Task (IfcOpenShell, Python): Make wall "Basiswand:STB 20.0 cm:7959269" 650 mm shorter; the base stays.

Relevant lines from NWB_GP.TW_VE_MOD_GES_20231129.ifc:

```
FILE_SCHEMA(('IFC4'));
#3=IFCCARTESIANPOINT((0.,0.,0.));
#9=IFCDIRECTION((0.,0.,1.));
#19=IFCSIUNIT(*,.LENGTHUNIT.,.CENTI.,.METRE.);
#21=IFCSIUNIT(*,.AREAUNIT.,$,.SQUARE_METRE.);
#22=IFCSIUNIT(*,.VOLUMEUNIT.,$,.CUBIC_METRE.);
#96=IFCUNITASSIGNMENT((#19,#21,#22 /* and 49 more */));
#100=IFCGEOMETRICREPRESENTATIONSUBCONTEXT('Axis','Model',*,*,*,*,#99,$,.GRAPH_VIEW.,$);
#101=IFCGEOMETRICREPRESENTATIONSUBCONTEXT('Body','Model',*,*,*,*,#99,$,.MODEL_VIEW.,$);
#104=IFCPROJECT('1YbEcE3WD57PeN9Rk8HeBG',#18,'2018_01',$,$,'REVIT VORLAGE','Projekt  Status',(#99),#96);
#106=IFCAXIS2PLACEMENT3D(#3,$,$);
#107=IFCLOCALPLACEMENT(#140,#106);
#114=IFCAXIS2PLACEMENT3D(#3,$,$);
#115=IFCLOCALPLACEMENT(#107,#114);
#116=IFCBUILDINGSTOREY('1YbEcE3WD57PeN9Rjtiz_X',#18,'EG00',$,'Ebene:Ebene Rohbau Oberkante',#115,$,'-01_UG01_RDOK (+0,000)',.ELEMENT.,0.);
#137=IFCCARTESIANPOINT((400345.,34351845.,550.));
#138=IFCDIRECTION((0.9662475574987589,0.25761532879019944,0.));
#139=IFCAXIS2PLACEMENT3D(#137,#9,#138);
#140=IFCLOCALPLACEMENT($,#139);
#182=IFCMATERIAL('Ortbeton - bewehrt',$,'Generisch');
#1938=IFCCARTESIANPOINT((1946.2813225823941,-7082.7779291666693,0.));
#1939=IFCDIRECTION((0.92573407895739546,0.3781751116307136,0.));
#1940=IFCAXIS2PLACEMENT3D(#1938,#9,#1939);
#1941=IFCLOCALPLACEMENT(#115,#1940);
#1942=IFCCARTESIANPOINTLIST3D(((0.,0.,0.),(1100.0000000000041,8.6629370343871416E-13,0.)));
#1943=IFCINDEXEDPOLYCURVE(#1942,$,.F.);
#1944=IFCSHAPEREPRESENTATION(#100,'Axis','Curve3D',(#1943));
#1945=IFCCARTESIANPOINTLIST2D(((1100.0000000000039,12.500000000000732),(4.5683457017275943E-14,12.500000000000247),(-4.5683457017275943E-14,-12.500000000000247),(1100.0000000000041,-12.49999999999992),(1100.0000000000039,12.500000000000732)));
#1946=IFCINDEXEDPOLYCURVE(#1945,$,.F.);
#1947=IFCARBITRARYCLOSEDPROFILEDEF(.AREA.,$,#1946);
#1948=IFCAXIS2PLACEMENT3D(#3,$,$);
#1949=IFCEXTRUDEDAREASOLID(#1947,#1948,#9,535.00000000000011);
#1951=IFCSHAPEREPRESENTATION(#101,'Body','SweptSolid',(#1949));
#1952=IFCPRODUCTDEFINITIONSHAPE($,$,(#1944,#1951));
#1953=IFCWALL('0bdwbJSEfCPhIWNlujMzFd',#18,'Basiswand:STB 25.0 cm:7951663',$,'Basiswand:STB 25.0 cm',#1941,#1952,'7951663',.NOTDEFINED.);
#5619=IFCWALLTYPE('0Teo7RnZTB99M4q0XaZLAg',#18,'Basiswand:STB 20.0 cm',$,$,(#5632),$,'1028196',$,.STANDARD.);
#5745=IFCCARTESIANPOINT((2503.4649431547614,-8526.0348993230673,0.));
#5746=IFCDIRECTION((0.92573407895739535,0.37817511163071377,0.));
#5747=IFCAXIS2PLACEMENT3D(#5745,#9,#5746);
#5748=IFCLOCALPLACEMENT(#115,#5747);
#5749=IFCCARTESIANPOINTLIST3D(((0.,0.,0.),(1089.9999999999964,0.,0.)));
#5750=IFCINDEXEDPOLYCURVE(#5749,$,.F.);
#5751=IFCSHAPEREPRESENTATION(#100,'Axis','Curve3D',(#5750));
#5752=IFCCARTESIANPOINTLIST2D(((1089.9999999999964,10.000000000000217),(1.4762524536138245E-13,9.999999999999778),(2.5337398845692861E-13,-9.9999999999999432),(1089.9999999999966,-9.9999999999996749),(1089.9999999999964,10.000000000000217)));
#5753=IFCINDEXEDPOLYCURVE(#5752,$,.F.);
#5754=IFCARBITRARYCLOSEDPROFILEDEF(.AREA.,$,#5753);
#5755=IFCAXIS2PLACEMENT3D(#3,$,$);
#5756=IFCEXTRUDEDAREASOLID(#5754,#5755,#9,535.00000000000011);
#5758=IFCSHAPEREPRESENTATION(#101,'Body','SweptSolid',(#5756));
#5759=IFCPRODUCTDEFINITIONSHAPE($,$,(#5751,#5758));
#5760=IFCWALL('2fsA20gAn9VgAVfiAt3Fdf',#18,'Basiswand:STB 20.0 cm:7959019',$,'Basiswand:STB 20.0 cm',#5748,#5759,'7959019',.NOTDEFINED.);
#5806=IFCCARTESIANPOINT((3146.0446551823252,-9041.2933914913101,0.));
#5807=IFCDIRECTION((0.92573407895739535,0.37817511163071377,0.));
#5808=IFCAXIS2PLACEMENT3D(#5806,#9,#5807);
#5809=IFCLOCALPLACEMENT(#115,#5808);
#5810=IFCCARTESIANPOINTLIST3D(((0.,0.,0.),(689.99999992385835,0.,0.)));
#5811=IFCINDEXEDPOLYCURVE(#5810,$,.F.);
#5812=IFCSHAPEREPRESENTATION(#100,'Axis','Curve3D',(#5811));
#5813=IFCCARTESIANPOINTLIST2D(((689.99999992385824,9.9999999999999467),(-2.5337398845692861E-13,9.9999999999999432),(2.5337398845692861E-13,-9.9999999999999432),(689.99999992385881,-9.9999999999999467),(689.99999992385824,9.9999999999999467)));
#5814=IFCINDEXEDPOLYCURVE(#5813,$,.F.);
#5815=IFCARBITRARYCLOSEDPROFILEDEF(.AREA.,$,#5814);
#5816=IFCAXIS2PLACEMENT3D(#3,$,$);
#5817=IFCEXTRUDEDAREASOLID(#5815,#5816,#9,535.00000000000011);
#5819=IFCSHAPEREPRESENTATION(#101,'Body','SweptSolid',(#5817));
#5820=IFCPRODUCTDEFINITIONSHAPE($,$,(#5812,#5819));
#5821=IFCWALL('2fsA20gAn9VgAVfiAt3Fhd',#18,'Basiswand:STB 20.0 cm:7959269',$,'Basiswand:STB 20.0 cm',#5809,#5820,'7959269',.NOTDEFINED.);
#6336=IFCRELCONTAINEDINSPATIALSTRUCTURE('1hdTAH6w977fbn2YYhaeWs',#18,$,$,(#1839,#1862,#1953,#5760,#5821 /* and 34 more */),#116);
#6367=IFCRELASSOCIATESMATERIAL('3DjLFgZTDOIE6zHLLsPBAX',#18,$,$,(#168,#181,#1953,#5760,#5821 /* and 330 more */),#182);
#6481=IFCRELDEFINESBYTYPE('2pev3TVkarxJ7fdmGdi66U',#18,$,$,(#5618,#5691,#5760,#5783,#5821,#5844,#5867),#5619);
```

```python
import ifcopenshell
import ifcopenshell.geom
import ifcopenshell.util.representation
import ifcopenshell.util.shape
import ifcopenshell.util.unit

model = ifcopenshell.open("NWB_GP.TW_VE_MOD_GES_20231129.ifc")
unit_scale = ifcopenshell.util.unit.calculate_unit_scale(model)
settings = ifcopenshell.geom.settings()


def volume(element):
    """Net volume in cubic metres, openings subtracted."""
    shape = ifcopenshell.geom.create_shape(settings, element)
    return ifcopenshell.util.shape.get_volume(shape.geometry)


wall = model.by_guid("2fsA20gAn9VgAVfiAt3Fhd")
before = volume(wall)

body = ifcopenshell.util.representation.get_representation(wall, "Model", "Body")
solid = body.Items[0]
old_height = solid.Depth
solid.Depth -= 0.65 / unit_scale
after = volume(wall)

print(f"height {old_height:g} -> {solid.Depth:g}, volume {before:.3f} -> {after:.3f} m3")

model.write("NWB_GP.TW_VE_MOD_GES_20231129_v2.ifc")
```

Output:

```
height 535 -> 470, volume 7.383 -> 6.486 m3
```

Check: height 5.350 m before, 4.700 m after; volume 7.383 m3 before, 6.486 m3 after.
